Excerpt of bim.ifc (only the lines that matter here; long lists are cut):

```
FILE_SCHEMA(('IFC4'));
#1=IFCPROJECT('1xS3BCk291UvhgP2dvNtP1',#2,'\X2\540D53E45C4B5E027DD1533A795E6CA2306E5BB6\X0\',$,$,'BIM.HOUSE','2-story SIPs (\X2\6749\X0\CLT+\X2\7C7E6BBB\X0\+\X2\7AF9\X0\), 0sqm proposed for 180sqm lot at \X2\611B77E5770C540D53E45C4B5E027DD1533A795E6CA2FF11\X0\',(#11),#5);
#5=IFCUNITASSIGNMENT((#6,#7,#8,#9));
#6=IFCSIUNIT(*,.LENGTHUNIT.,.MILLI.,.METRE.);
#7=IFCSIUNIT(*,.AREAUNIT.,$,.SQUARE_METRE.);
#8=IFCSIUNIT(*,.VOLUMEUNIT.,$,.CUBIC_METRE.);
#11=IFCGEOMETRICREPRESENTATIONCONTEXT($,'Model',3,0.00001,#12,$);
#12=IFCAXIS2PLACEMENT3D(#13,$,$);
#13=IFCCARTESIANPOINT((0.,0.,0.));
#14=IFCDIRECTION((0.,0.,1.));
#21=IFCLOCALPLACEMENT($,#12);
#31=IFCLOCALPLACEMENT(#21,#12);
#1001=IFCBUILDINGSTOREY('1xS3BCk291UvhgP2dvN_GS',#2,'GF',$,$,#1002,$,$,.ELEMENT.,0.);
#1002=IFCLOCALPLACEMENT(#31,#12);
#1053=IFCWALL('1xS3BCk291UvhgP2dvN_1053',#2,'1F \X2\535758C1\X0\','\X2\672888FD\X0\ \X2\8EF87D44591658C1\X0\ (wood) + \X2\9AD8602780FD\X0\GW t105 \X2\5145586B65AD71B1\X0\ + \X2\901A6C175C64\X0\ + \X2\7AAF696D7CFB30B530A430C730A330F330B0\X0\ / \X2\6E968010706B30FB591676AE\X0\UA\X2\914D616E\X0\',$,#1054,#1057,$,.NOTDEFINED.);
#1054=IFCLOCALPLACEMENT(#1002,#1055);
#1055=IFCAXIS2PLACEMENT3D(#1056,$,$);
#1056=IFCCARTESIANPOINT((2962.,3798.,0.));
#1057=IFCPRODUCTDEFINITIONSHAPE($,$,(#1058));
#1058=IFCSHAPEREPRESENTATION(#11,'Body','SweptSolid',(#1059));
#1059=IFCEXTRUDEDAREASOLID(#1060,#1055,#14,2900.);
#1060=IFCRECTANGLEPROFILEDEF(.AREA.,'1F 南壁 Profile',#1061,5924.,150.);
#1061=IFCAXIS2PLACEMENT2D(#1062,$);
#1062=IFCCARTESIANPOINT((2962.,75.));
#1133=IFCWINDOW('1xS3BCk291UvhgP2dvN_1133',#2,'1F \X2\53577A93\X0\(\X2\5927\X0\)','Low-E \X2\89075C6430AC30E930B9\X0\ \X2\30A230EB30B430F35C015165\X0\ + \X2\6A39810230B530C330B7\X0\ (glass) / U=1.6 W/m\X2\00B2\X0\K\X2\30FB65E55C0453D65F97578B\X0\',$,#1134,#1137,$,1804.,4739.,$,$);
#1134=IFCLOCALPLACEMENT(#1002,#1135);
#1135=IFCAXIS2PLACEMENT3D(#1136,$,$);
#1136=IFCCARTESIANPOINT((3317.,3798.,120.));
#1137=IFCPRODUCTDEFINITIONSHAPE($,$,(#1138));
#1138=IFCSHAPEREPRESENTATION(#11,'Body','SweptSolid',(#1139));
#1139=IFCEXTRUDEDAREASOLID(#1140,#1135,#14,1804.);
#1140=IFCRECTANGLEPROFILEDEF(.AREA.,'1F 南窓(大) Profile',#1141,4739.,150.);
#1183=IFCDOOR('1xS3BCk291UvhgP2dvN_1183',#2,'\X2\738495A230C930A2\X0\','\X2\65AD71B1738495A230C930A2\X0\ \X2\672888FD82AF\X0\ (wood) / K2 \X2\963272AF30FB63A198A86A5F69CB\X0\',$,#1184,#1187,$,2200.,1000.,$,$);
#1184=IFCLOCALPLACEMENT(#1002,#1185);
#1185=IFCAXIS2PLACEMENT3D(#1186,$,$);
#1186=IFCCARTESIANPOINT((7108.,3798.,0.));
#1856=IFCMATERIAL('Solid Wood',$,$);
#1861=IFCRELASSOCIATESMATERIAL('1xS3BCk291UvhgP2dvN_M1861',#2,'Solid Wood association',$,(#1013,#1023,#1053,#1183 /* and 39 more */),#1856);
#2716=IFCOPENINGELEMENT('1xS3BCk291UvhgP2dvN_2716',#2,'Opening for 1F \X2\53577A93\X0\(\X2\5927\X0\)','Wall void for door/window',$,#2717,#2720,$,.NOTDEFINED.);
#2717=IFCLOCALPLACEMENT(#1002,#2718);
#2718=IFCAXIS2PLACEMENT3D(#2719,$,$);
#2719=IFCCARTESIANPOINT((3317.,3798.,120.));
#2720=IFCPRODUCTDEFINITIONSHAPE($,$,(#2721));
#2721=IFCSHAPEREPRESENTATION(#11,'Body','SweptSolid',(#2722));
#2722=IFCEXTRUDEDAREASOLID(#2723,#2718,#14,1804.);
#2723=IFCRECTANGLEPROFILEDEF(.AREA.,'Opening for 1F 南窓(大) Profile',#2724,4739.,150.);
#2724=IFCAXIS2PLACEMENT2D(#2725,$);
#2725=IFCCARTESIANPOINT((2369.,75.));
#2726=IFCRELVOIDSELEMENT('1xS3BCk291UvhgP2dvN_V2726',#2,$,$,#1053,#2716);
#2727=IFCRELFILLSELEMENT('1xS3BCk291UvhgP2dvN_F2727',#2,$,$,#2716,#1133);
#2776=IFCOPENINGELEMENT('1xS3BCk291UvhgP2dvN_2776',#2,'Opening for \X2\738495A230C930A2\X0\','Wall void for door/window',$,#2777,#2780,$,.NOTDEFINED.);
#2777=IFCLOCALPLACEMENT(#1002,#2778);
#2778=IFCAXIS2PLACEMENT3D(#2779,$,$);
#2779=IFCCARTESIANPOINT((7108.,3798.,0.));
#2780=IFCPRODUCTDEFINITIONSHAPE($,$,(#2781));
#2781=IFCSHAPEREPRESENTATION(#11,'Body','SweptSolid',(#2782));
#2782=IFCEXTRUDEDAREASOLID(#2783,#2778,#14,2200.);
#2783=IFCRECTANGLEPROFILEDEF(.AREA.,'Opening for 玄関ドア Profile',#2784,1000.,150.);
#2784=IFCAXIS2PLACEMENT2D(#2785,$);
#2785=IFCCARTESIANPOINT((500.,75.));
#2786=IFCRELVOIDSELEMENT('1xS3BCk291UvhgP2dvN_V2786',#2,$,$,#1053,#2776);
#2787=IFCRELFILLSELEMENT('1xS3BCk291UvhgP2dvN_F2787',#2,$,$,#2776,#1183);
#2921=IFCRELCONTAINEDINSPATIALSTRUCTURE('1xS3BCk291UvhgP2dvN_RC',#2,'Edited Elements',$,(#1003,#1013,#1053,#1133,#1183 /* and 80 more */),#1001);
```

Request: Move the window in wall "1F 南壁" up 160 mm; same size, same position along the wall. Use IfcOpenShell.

```python
import numpy as np
import ifcopenshell
import ifcopenshell.api.geometry
import ifcopenshell.util.placement
import ifcopenshell.util.unit

model = ifcopenshell.open("bim.ifc")
unit_scale = ifcopenshell.util.unit.calculate_unit_scale(model)

window = model.by_guid("1xS3BCk291UvhgP2dvN_1133")
opening = window.FillsVoids[0].RelatingOpeningElement
dz = 0.16 / unit_scale

shift = np.array([0.0, 0.0, dz])
# The window is not placed relative to its opening, so move both.
for product in (opening, window):
    matrix = ifcopenshell.util.placement.get_local_placement(product.ObjectPlacement)
    matrix[:3, 3] += shift
    ifcopenshell.api.geometry.edit_object_placement(model, product=product, matrix=matrix, is_si=False)

print(f"moved by {dz * unit_scale:+.3f} m")

model.write("bim_edited.ifc")
```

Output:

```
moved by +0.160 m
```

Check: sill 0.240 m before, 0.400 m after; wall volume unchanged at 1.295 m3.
